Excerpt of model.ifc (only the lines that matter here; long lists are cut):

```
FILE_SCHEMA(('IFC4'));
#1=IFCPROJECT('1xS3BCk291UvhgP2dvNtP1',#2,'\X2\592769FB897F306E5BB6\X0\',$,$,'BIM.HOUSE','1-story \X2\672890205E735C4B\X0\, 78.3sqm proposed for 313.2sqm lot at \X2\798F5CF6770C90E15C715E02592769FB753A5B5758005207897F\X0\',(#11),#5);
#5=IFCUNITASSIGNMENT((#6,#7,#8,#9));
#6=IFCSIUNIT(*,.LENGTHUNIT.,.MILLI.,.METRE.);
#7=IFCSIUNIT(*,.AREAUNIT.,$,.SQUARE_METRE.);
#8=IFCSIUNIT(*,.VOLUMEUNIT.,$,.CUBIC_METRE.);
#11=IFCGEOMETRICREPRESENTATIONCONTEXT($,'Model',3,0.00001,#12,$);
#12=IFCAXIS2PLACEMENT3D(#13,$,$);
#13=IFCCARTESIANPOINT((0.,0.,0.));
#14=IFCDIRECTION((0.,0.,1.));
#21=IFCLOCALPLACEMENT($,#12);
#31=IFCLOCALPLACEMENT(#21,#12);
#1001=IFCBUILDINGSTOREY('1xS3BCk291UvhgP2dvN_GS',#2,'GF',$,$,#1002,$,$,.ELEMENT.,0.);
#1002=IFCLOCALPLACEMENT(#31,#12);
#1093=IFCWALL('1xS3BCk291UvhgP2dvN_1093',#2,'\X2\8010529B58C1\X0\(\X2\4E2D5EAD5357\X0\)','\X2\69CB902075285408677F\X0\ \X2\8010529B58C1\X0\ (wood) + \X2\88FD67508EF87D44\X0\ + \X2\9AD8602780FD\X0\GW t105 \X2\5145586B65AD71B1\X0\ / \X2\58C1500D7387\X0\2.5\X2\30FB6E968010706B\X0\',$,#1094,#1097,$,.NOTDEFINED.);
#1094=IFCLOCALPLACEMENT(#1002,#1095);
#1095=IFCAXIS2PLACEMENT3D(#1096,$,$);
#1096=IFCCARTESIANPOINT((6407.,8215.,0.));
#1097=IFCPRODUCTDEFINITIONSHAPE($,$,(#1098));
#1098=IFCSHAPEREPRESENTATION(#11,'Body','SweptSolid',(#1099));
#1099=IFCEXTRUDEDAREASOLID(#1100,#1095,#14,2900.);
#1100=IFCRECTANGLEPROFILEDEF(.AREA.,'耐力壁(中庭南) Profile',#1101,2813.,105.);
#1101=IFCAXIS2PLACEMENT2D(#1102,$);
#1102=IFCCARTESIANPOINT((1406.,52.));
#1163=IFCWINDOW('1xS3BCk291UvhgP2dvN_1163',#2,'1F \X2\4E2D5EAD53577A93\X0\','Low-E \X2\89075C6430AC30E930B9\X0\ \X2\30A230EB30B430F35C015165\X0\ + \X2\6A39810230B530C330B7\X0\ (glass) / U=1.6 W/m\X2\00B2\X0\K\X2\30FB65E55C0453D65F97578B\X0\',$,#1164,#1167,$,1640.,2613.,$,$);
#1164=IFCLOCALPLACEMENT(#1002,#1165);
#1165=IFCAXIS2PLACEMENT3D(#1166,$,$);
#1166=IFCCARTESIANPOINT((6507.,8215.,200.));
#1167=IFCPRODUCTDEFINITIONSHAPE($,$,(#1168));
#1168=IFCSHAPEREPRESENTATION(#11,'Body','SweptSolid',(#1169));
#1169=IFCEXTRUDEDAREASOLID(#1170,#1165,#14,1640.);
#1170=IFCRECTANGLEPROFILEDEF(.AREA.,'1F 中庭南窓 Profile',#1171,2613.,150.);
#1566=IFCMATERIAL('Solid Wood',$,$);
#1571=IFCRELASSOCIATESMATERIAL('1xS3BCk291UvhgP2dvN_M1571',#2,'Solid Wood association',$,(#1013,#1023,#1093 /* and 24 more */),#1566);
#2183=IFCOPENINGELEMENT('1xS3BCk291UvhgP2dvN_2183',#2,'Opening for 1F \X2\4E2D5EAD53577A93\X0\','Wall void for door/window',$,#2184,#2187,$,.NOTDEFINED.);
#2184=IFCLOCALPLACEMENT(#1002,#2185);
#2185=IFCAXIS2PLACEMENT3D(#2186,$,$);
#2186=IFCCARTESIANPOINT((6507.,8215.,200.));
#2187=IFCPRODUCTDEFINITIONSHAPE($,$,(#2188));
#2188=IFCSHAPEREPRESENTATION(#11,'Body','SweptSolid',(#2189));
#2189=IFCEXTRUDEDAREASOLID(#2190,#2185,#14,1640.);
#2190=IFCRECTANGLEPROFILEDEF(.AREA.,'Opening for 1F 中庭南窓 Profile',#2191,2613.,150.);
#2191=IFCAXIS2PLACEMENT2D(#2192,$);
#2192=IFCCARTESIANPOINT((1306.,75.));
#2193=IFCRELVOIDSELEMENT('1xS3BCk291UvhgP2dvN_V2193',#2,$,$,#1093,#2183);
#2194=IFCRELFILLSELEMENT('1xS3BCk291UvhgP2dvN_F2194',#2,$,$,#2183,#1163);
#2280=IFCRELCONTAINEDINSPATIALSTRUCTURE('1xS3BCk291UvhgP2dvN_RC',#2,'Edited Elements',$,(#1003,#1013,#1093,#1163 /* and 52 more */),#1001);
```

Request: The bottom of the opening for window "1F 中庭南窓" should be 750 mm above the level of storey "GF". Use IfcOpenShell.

```python
import numpy as np
import ifcopenshell
import ifcopenshell.api.geometry
import ifcopenshell.geom
import ifcopenshell.util.element
import ifcopenshell.util.placement
import ifcopenshell.util.shape
import ifcopenshell.util.unit

model = ifcopenshell.open("model.ifc")
unit_scale = ifcopenshell.util.unit.calculate_unit_scale(model)

window = model.by_guid("1xS3BCk291UvhgP2dvN_1163")
opening = window.FillsVoids[0].RelatingOpeningElement
storey = ifcopenshell.util.element.get_container(window, ifc_class="IfcBuildingStorey")
level = ifcopenshell.util.placement.get_local_placement(storey.ObjectPlacement)[2, 3]

# The opening's origin need not be at the sill, so measure its lowest point.
shape = ifcopenshell.geom.create_shape(ifcopenshell.geom.settings(), opening)
bottom = ifcopenshell.util.shape.get_shape_bottom_elevation(shape, shape.geometry) / unit_scale
dz = level + 0.75 / unit_scale - bottom

shift = np.array([0.0, 0.0, dz])
# The window is not placed relative to its opening, so move both.
for product in (opening, window):
    matrix = ifcopenshell.util.placement.get_local_placement(product.ObjectPlacement)
    matrix[:3, 3] += shift
    ifcopenshell.api.geometry.edit_object_placement(model, product=product, matrix=matrix, is_si=False)

print(f"moved by {dz * unit_scale:+.3f} m")

model.write("model_rev.ifc")
```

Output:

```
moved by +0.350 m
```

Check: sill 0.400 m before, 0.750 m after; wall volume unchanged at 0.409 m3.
